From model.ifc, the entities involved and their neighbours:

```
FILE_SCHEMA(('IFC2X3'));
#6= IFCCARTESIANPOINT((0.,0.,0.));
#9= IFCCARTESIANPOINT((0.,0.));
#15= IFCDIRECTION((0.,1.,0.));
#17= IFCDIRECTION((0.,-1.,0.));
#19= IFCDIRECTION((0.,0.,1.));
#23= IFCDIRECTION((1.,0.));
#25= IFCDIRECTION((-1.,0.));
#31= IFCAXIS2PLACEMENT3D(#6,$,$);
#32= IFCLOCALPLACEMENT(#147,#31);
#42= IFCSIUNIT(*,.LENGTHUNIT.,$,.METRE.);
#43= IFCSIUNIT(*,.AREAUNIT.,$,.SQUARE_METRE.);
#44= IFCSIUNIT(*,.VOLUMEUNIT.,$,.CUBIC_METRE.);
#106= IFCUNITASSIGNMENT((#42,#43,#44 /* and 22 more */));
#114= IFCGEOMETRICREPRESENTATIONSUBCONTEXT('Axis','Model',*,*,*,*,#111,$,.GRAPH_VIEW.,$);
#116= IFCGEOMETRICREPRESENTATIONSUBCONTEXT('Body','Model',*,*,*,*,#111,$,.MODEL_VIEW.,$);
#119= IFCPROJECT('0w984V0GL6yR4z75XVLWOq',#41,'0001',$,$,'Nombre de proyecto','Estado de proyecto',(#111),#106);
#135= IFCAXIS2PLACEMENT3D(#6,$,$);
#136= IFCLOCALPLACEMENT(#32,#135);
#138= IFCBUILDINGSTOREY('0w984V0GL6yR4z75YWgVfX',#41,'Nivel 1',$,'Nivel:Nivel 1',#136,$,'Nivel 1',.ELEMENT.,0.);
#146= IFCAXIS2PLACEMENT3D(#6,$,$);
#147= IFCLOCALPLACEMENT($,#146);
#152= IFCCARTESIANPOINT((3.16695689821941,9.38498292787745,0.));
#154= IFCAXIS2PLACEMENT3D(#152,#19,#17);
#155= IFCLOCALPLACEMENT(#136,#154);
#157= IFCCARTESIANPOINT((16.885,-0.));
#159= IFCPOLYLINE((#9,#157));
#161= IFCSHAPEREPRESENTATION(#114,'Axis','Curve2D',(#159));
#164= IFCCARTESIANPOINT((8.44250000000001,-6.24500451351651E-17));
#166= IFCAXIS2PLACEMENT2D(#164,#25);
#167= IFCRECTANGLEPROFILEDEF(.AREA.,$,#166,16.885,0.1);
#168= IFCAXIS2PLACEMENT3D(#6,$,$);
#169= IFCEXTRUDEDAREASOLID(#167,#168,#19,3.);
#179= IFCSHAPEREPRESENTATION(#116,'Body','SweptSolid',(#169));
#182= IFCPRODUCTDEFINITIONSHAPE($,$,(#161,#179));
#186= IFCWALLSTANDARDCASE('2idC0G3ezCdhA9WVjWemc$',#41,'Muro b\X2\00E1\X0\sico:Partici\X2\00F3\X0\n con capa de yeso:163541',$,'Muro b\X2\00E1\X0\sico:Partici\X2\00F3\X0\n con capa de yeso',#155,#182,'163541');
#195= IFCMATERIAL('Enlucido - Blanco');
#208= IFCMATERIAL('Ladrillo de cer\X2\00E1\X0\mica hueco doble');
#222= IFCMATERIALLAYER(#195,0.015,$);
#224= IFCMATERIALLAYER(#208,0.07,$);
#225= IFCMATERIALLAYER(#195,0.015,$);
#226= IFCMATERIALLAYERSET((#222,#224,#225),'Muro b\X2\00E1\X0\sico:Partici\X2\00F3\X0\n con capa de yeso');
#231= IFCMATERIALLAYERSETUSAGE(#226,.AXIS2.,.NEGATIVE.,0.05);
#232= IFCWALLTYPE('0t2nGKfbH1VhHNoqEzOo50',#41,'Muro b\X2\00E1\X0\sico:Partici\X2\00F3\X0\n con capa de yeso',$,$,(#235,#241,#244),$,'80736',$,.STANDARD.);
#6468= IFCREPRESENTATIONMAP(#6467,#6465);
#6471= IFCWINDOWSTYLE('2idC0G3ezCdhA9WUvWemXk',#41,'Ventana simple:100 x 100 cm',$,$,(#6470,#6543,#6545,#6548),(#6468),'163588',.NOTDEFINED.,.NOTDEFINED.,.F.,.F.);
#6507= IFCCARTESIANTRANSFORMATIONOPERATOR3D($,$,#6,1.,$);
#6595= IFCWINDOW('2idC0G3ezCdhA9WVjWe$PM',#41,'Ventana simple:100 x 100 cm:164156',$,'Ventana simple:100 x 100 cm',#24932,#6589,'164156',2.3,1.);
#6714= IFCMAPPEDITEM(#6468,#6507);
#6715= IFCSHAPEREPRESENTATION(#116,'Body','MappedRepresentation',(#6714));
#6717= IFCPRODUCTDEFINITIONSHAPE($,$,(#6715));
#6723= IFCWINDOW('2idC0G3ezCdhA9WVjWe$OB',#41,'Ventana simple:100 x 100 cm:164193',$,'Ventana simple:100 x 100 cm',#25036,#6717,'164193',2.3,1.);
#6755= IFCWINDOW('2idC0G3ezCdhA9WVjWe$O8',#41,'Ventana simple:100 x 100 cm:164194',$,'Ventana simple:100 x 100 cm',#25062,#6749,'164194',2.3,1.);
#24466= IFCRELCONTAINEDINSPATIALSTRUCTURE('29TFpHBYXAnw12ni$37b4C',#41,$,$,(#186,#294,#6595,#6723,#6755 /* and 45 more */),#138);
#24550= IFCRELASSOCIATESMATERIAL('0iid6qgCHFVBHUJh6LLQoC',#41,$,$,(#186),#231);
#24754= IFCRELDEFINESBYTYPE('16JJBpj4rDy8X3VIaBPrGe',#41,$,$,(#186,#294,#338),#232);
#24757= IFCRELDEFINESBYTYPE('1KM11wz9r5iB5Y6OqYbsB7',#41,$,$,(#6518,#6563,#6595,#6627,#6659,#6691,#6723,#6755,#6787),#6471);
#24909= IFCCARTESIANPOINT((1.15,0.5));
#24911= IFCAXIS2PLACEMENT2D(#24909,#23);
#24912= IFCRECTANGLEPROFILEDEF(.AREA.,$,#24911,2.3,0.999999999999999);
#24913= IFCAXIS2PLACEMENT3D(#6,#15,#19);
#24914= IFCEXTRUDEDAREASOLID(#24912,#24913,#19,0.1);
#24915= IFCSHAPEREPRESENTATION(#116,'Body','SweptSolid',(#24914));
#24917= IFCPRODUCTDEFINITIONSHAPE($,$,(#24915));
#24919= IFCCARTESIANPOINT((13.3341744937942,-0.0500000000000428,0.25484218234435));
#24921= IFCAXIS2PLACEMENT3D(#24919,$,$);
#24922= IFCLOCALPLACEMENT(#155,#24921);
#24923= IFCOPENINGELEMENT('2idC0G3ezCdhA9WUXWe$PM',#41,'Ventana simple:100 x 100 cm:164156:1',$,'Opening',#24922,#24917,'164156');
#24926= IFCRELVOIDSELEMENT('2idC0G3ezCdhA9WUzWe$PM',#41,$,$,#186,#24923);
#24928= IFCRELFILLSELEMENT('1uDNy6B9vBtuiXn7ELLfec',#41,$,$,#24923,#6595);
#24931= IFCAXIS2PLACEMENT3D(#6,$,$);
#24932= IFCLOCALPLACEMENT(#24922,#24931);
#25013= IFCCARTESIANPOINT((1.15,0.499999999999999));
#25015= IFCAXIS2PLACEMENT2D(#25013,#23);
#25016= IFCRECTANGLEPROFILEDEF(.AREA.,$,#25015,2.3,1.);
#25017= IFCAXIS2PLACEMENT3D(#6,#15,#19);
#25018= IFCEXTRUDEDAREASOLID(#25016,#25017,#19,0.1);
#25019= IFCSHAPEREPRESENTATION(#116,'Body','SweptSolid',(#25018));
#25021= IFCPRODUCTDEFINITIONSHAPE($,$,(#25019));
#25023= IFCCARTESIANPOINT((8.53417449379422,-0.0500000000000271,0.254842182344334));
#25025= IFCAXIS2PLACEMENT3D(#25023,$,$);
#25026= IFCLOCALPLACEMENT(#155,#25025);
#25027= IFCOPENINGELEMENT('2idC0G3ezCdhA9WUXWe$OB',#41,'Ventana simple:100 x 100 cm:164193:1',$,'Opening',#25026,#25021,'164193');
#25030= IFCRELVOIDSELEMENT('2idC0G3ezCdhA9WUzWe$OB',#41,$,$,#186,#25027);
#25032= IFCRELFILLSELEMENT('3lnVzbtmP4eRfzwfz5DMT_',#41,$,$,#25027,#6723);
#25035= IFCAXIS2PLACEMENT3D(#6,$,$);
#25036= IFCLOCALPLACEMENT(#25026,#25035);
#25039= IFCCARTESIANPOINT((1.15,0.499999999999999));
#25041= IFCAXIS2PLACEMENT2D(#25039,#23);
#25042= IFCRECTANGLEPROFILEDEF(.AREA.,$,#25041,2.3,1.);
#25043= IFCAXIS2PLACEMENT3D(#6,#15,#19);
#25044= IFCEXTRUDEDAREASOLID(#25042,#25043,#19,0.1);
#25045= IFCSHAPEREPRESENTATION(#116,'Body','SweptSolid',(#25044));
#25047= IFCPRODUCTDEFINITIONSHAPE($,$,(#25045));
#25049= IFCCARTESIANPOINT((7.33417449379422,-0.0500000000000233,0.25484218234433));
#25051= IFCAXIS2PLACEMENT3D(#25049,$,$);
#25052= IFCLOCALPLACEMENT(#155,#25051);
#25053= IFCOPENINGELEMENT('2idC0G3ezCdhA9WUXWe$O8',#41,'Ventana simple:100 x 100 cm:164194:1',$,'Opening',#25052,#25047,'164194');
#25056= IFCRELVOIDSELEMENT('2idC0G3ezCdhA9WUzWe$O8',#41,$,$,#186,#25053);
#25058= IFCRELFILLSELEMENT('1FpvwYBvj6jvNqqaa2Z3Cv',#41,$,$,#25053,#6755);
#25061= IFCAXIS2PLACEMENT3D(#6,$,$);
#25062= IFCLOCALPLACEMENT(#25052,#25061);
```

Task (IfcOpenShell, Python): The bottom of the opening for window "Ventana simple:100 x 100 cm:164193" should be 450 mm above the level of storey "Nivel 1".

```python
import numpy as np
import ifcopenshell
import ifcopenshell.api.geometry
import ifcopenshell.geom
import ifcopenshell.util.element
import ifcopenshell.util.placement
import ifcopenshell.util.shape
import ifcopenshell.util.unit

model = ifcopenshell.open("model.ifc")
unit_scale = ifcopenshell.util.unit.calculate_unit_scale(model)

window = model.by_id(6723)
opening = window.FillsVoids[0].RelatingOpeningElement
storey = ifcopenshell.util.element.get_container(window, ifc_class="IfcBuildingStorey")
level = ifcopenshell.util.placement.get_local_placement(storey.ObjectPlacement)[2, 3]

# The opening's origin need not be at the sill, so measure its lowest point.
shape = ifcopenshell.geom.create_shape(ifcopenshell.geom.settings(), opening)
bottom = ifcopenshell.util.shape.get_shape_bottom_elevation(shape, shape.geometry) / unit_scale
dz = level + 0.45 - bottom

shift = np.array([0.0, 0.0, dz])
# The window is placed relative to its opening, so it follows when the opening moves.
matrix = ifcopenshell.util.placement.get_local_placement(opening.ObjectPlacement)
matrix[:3, 3] += shift
ifcopenshell.api.geometry.edit_object_placement(
    model, product=opening, matrix=matrix, is_si=False, should_transform_children=True
)

print(f"moved by {dz * unit_scale:+.3f} m")

model.write("model_edited.ifc")
```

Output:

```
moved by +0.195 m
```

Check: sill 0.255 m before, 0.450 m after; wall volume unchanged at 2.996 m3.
